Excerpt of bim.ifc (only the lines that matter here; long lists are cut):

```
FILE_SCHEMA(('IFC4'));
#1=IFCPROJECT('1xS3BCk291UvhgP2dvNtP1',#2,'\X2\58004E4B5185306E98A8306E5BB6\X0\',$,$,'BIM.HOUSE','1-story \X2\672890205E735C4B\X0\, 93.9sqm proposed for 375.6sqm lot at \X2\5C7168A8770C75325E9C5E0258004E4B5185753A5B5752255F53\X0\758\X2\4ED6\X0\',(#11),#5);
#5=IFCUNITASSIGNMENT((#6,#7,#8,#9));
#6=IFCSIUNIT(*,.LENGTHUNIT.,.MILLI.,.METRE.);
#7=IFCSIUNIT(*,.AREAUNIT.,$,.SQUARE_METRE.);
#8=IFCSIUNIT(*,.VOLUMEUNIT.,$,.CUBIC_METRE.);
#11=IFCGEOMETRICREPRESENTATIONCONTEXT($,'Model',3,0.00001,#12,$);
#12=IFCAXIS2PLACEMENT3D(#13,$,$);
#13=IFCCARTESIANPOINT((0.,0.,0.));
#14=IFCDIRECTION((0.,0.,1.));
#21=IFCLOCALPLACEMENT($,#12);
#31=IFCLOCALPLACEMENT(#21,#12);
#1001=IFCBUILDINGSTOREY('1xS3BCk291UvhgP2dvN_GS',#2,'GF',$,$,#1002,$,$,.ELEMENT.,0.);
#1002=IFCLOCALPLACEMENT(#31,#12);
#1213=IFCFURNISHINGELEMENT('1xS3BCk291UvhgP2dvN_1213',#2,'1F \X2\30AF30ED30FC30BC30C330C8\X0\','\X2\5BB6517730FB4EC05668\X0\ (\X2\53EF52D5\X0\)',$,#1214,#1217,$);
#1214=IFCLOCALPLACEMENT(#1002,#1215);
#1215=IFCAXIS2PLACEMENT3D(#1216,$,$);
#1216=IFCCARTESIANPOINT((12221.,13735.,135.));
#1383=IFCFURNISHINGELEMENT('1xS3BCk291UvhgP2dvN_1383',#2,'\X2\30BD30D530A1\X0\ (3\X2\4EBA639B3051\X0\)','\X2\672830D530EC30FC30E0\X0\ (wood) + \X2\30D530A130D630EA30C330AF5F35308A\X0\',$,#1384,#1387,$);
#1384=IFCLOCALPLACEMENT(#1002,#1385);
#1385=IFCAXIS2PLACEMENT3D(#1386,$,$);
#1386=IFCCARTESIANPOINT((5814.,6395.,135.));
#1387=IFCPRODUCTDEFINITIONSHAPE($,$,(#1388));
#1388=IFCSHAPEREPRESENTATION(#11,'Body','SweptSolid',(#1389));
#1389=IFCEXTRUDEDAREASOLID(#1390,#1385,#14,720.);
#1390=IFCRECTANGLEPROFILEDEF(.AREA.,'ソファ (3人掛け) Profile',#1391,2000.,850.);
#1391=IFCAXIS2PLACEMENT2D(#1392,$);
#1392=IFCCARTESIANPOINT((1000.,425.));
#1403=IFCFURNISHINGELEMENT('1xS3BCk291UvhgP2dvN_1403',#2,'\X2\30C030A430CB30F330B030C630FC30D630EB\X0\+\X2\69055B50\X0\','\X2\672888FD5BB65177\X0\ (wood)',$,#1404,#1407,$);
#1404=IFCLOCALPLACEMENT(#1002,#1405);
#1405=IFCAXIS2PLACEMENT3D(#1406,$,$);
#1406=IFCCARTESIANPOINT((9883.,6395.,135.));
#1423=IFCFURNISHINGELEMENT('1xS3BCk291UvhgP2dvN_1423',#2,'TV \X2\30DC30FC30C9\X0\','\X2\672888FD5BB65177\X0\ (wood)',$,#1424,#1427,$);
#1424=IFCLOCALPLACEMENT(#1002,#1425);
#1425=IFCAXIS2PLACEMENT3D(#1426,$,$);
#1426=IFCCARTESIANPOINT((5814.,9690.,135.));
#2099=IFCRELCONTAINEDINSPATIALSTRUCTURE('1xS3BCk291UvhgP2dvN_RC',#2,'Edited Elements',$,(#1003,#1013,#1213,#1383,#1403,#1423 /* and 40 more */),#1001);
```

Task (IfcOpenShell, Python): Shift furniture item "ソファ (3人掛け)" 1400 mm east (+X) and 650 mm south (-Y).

```python
import ifcopenshell
import ifcopenshell.api.geometry
import ifcopenshell.util.placement

model = ifcopenshell.open("bim.ifc")

item = model.by_guid("1xS3BCk291UvhgP2dvN_1383")
matrix = ifcopenshell.util.placement.get_local_placement(item.ObjectPlacement)
matrix[0, 3] += 1400.0
matrix[1, 3] -= 650.0
ifcopenshell.api.geometry.edit_object_placement(model, product=item, matrix=matrix, is_si=False)

print(ifcopenshell.util.placement.get_local_placement(item.ObjectPlacement).round(3) + 0.0)

model.write("bim-out.ifc")
```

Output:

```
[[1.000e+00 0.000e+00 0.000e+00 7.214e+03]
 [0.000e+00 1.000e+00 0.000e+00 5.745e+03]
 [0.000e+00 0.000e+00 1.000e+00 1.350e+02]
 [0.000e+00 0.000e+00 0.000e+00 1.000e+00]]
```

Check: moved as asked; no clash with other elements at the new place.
